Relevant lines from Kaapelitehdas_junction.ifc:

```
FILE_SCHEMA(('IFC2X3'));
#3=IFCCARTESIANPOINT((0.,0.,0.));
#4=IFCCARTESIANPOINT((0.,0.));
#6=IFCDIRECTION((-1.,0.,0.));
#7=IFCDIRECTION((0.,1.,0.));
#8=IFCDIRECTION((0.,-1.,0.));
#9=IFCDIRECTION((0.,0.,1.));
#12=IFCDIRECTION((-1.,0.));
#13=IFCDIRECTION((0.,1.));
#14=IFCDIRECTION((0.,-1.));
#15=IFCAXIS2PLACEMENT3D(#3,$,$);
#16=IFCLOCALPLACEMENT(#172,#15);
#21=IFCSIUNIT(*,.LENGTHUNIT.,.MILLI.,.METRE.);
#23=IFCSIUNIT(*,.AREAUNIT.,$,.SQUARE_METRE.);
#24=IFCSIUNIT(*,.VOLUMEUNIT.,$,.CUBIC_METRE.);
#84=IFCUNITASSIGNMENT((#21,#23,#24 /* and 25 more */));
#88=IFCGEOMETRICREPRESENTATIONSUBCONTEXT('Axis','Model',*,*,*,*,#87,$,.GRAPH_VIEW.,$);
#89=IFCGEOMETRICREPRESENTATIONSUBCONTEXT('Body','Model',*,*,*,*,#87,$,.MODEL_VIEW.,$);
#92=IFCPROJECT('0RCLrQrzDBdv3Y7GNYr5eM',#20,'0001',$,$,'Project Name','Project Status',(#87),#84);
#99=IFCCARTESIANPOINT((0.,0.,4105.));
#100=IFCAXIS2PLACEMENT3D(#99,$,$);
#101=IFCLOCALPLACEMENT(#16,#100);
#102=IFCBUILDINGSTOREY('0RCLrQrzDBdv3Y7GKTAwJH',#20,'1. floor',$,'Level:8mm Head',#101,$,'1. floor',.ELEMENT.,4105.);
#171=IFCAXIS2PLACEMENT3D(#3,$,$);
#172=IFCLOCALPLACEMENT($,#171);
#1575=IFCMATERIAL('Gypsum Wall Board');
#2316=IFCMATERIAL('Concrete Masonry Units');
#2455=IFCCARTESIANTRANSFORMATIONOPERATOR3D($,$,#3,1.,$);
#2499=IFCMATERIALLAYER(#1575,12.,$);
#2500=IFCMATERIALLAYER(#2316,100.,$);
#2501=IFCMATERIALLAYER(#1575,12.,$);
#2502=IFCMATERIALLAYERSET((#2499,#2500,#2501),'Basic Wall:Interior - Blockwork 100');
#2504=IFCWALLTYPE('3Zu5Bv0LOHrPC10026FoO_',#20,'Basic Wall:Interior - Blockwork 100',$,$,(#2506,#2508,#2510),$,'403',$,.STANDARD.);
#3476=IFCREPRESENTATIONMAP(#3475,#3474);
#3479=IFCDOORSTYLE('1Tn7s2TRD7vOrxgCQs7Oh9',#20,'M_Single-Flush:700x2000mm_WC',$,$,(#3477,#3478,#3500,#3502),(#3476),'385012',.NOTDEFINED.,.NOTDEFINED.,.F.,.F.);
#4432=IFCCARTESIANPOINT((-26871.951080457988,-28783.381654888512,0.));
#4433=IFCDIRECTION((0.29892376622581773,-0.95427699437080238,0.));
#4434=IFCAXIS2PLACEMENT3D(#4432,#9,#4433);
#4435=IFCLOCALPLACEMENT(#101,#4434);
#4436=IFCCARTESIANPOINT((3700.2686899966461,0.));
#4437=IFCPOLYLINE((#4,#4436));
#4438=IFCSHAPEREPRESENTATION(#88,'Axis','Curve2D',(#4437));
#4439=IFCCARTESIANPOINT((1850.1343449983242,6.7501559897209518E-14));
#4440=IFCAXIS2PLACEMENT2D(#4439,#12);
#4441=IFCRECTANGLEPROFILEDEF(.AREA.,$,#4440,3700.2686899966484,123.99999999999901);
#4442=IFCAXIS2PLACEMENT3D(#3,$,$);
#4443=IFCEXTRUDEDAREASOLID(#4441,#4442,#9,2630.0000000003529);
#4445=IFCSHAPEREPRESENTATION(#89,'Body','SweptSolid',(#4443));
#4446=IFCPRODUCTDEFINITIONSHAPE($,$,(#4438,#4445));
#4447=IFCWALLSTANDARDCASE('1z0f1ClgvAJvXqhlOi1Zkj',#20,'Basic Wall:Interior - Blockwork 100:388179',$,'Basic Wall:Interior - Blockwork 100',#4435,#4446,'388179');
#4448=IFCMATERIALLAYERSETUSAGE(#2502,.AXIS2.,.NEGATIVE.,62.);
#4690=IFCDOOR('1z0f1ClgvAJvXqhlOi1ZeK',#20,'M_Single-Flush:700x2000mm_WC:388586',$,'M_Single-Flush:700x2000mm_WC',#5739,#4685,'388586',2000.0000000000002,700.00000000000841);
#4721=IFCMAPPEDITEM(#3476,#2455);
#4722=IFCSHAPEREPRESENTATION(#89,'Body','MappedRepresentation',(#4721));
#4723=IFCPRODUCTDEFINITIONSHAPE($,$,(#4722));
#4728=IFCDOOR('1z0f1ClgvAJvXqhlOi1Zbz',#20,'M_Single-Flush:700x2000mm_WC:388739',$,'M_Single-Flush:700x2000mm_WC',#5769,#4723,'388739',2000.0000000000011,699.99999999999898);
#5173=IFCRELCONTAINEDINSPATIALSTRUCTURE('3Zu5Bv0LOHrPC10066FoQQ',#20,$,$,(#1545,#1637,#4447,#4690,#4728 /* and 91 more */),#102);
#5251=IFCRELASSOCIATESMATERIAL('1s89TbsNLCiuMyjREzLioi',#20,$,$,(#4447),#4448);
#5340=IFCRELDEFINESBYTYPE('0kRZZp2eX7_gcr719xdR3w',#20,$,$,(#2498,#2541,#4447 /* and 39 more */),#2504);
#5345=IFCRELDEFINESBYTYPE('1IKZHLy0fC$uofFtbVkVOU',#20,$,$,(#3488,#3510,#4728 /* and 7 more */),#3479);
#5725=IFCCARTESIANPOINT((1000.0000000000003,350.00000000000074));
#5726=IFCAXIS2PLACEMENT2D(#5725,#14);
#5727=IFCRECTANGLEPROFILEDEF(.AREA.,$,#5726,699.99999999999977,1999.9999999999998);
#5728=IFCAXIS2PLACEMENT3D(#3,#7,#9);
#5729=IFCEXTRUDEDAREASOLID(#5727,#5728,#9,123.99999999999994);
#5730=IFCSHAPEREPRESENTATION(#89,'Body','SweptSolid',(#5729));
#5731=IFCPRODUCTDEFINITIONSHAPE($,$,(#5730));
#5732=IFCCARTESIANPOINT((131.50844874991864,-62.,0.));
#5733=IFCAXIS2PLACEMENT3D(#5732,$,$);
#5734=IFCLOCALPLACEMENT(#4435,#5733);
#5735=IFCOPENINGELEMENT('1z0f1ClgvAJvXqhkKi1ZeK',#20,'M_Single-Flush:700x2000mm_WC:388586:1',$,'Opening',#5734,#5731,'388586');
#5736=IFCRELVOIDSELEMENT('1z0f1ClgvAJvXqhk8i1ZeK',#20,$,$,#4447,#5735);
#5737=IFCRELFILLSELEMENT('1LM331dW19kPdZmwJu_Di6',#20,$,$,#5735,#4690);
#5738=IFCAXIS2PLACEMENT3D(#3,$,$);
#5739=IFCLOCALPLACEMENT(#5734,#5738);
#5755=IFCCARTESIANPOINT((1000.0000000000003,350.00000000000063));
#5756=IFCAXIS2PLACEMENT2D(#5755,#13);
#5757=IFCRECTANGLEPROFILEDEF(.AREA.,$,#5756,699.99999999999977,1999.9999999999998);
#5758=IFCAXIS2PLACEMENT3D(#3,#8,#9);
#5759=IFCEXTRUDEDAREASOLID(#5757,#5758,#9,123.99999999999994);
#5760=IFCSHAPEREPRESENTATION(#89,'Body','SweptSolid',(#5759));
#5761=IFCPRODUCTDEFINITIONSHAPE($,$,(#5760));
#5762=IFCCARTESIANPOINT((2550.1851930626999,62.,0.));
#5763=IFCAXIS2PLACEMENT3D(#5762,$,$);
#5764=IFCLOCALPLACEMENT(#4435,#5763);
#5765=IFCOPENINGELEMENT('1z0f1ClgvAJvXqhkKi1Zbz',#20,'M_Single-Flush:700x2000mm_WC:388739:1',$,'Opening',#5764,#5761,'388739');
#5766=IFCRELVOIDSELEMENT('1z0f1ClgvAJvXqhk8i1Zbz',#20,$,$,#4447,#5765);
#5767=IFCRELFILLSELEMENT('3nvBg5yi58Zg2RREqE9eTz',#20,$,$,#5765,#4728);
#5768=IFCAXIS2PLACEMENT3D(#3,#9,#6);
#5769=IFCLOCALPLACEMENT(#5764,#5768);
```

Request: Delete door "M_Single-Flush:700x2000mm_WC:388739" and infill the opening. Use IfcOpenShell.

```python
import ifcopenshell
import ifcopenshell.api.feature
import ifcopenshell.api.root
import ifcopenshell.geom
import ifcopenshell.util.shape

model = ifcopenshell.open("Kaapelitehdas_junction.ifc")
settings = ifcopenshell.geom.settings()


def volume(element):
    """Net volume in cubic metres, openings subtracted."""
    shape = ifcopenshell.geom.create_shape(settings, element)
    return ifcopenshell.util.shape.get_volume(shape.geometry)


door = model.by_guid("1z0f1ClgvAJvXqhlOi1Zbz")
opening = door.FillsVoids[0].RelatingOpeningElement
wall = opening.VoidsElements[0].RelatingBuildingElement
before = volume(wall)

ifcopenshell.api.root.remove_product(model, product=door)
ifcopenshell.api.feature.remove_feature(model, feature=opening)

after = volume(wall)

print(f"wall volume {before:.3f} -> {after:.3f} m3")

model.write("Kaapelitehdas_junction-out.ifc")
```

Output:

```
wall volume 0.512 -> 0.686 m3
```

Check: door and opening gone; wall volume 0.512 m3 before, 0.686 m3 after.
